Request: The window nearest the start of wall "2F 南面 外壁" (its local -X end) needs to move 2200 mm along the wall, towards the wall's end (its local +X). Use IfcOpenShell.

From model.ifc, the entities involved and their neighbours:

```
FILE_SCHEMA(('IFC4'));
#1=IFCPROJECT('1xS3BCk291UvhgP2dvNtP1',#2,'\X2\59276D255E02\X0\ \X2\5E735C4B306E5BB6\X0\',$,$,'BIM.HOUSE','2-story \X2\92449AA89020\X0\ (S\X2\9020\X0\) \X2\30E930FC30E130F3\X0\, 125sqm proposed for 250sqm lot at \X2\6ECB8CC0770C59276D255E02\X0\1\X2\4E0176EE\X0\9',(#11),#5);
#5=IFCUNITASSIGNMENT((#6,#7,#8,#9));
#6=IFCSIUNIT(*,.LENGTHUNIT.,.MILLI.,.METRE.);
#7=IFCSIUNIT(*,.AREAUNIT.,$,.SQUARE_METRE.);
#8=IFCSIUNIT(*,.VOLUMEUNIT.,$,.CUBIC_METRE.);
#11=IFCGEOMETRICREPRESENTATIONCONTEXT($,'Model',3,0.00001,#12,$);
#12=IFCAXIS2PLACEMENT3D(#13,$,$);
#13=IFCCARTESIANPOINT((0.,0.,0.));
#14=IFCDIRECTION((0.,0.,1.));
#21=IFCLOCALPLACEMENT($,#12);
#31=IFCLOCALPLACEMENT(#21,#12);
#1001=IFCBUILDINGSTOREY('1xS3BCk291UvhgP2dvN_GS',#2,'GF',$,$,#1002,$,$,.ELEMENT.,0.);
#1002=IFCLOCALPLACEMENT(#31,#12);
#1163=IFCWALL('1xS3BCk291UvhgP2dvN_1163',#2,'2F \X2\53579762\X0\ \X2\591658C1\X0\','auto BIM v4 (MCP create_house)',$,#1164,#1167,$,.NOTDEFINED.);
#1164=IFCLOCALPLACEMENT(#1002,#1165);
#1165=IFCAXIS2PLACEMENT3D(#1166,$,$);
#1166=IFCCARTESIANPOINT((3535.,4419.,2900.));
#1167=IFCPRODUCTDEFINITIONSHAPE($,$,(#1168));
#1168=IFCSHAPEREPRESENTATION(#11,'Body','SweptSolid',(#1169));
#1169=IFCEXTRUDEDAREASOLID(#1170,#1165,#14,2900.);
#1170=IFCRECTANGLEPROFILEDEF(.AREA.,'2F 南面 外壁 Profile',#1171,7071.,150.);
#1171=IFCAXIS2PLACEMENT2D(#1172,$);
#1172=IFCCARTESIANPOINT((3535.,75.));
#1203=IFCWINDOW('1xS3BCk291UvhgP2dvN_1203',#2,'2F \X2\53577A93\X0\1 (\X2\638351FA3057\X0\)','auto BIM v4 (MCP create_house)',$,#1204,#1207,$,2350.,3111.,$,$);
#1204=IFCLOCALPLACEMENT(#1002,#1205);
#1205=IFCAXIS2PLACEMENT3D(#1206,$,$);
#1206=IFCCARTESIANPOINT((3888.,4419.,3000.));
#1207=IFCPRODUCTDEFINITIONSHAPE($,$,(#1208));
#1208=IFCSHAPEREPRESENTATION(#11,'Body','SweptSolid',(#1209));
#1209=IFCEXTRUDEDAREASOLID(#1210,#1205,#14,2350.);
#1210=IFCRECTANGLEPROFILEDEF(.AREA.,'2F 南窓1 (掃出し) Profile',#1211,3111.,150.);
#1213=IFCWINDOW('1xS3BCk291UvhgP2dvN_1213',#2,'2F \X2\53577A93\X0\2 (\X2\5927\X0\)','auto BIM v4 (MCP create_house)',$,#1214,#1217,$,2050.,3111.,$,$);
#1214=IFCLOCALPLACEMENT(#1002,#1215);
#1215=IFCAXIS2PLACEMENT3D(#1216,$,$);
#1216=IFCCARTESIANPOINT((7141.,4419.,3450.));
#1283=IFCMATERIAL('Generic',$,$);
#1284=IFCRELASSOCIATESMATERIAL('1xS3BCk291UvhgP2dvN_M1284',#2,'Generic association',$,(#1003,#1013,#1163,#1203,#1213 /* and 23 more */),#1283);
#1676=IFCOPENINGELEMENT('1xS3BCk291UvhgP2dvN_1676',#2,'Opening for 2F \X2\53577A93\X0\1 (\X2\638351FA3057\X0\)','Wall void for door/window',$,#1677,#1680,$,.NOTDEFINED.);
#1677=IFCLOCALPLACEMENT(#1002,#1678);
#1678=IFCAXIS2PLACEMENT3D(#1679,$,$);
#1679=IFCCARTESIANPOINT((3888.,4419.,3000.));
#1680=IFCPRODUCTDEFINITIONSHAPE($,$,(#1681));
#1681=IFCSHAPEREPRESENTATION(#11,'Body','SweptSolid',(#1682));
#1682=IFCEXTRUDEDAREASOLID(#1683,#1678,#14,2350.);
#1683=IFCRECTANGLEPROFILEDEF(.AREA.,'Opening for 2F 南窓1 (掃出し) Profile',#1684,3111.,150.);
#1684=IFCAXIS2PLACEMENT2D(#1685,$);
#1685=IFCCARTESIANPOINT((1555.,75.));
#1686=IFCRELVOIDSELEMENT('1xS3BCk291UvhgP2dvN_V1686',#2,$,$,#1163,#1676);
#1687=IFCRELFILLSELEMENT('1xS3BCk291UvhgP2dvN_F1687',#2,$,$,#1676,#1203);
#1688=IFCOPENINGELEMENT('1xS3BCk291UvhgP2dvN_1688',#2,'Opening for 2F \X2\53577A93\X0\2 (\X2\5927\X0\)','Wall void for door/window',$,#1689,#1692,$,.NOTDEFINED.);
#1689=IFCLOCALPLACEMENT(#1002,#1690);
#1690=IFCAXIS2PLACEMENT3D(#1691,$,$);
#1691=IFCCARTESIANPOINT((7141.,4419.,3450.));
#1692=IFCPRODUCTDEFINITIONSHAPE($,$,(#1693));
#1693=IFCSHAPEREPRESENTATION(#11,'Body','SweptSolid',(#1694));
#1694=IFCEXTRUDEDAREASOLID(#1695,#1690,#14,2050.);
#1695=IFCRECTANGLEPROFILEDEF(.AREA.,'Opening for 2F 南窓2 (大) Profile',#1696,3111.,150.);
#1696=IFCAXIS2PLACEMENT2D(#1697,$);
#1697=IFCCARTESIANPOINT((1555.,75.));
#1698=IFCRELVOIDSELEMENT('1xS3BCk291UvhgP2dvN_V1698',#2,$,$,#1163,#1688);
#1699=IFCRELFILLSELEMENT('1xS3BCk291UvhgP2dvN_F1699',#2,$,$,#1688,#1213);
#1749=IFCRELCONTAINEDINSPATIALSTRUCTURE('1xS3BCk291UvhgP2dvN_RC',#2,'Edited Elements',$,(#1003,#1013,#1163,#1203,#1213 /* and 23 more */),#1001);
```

```python
import ifcopenshell
import ifcopenshell.api.geometry
import ifcopenshell.util.placement

model = ifcopenshell.open("model.ifc")

window = model.by_id(1203)
opening = window.FillsVoids[0].RelatingOpeningElement
wall = opening.VoidsElements[0].RelatingBuildingElement

wall_matrix = ifcopenshell.util.placement.get_local_placement(wall.ObjectPlacement)
shift = wall_matrix[:3, 0] * 2200.0
before = ifcopenshell.util.placement.get_local_placement(window.ObjectPlacement)[:3, 3].copy()

# The window is not placed relative to its opening, so move both.
for product in (opening, window):
    matrix = ifcopenshell.util.placement.get_local_placement(product.ObjectPlacement)
    matrix[:3, 3] += shift
    ifcopenshell.api.geometry.edit_object_placement(model, product=product, matrix=matrix, is_si=False)

after = ifcopenshell.util.placement.get_local_placement(window.ObjectPlacement)[:3, 3]
print("window moved by", (after - before).round(3) + 0.0)

model.write("model-out.ifc")
```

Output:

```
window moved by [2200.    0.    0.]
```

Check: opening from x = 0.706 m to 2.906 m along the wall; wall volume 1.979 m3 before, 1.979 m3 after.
